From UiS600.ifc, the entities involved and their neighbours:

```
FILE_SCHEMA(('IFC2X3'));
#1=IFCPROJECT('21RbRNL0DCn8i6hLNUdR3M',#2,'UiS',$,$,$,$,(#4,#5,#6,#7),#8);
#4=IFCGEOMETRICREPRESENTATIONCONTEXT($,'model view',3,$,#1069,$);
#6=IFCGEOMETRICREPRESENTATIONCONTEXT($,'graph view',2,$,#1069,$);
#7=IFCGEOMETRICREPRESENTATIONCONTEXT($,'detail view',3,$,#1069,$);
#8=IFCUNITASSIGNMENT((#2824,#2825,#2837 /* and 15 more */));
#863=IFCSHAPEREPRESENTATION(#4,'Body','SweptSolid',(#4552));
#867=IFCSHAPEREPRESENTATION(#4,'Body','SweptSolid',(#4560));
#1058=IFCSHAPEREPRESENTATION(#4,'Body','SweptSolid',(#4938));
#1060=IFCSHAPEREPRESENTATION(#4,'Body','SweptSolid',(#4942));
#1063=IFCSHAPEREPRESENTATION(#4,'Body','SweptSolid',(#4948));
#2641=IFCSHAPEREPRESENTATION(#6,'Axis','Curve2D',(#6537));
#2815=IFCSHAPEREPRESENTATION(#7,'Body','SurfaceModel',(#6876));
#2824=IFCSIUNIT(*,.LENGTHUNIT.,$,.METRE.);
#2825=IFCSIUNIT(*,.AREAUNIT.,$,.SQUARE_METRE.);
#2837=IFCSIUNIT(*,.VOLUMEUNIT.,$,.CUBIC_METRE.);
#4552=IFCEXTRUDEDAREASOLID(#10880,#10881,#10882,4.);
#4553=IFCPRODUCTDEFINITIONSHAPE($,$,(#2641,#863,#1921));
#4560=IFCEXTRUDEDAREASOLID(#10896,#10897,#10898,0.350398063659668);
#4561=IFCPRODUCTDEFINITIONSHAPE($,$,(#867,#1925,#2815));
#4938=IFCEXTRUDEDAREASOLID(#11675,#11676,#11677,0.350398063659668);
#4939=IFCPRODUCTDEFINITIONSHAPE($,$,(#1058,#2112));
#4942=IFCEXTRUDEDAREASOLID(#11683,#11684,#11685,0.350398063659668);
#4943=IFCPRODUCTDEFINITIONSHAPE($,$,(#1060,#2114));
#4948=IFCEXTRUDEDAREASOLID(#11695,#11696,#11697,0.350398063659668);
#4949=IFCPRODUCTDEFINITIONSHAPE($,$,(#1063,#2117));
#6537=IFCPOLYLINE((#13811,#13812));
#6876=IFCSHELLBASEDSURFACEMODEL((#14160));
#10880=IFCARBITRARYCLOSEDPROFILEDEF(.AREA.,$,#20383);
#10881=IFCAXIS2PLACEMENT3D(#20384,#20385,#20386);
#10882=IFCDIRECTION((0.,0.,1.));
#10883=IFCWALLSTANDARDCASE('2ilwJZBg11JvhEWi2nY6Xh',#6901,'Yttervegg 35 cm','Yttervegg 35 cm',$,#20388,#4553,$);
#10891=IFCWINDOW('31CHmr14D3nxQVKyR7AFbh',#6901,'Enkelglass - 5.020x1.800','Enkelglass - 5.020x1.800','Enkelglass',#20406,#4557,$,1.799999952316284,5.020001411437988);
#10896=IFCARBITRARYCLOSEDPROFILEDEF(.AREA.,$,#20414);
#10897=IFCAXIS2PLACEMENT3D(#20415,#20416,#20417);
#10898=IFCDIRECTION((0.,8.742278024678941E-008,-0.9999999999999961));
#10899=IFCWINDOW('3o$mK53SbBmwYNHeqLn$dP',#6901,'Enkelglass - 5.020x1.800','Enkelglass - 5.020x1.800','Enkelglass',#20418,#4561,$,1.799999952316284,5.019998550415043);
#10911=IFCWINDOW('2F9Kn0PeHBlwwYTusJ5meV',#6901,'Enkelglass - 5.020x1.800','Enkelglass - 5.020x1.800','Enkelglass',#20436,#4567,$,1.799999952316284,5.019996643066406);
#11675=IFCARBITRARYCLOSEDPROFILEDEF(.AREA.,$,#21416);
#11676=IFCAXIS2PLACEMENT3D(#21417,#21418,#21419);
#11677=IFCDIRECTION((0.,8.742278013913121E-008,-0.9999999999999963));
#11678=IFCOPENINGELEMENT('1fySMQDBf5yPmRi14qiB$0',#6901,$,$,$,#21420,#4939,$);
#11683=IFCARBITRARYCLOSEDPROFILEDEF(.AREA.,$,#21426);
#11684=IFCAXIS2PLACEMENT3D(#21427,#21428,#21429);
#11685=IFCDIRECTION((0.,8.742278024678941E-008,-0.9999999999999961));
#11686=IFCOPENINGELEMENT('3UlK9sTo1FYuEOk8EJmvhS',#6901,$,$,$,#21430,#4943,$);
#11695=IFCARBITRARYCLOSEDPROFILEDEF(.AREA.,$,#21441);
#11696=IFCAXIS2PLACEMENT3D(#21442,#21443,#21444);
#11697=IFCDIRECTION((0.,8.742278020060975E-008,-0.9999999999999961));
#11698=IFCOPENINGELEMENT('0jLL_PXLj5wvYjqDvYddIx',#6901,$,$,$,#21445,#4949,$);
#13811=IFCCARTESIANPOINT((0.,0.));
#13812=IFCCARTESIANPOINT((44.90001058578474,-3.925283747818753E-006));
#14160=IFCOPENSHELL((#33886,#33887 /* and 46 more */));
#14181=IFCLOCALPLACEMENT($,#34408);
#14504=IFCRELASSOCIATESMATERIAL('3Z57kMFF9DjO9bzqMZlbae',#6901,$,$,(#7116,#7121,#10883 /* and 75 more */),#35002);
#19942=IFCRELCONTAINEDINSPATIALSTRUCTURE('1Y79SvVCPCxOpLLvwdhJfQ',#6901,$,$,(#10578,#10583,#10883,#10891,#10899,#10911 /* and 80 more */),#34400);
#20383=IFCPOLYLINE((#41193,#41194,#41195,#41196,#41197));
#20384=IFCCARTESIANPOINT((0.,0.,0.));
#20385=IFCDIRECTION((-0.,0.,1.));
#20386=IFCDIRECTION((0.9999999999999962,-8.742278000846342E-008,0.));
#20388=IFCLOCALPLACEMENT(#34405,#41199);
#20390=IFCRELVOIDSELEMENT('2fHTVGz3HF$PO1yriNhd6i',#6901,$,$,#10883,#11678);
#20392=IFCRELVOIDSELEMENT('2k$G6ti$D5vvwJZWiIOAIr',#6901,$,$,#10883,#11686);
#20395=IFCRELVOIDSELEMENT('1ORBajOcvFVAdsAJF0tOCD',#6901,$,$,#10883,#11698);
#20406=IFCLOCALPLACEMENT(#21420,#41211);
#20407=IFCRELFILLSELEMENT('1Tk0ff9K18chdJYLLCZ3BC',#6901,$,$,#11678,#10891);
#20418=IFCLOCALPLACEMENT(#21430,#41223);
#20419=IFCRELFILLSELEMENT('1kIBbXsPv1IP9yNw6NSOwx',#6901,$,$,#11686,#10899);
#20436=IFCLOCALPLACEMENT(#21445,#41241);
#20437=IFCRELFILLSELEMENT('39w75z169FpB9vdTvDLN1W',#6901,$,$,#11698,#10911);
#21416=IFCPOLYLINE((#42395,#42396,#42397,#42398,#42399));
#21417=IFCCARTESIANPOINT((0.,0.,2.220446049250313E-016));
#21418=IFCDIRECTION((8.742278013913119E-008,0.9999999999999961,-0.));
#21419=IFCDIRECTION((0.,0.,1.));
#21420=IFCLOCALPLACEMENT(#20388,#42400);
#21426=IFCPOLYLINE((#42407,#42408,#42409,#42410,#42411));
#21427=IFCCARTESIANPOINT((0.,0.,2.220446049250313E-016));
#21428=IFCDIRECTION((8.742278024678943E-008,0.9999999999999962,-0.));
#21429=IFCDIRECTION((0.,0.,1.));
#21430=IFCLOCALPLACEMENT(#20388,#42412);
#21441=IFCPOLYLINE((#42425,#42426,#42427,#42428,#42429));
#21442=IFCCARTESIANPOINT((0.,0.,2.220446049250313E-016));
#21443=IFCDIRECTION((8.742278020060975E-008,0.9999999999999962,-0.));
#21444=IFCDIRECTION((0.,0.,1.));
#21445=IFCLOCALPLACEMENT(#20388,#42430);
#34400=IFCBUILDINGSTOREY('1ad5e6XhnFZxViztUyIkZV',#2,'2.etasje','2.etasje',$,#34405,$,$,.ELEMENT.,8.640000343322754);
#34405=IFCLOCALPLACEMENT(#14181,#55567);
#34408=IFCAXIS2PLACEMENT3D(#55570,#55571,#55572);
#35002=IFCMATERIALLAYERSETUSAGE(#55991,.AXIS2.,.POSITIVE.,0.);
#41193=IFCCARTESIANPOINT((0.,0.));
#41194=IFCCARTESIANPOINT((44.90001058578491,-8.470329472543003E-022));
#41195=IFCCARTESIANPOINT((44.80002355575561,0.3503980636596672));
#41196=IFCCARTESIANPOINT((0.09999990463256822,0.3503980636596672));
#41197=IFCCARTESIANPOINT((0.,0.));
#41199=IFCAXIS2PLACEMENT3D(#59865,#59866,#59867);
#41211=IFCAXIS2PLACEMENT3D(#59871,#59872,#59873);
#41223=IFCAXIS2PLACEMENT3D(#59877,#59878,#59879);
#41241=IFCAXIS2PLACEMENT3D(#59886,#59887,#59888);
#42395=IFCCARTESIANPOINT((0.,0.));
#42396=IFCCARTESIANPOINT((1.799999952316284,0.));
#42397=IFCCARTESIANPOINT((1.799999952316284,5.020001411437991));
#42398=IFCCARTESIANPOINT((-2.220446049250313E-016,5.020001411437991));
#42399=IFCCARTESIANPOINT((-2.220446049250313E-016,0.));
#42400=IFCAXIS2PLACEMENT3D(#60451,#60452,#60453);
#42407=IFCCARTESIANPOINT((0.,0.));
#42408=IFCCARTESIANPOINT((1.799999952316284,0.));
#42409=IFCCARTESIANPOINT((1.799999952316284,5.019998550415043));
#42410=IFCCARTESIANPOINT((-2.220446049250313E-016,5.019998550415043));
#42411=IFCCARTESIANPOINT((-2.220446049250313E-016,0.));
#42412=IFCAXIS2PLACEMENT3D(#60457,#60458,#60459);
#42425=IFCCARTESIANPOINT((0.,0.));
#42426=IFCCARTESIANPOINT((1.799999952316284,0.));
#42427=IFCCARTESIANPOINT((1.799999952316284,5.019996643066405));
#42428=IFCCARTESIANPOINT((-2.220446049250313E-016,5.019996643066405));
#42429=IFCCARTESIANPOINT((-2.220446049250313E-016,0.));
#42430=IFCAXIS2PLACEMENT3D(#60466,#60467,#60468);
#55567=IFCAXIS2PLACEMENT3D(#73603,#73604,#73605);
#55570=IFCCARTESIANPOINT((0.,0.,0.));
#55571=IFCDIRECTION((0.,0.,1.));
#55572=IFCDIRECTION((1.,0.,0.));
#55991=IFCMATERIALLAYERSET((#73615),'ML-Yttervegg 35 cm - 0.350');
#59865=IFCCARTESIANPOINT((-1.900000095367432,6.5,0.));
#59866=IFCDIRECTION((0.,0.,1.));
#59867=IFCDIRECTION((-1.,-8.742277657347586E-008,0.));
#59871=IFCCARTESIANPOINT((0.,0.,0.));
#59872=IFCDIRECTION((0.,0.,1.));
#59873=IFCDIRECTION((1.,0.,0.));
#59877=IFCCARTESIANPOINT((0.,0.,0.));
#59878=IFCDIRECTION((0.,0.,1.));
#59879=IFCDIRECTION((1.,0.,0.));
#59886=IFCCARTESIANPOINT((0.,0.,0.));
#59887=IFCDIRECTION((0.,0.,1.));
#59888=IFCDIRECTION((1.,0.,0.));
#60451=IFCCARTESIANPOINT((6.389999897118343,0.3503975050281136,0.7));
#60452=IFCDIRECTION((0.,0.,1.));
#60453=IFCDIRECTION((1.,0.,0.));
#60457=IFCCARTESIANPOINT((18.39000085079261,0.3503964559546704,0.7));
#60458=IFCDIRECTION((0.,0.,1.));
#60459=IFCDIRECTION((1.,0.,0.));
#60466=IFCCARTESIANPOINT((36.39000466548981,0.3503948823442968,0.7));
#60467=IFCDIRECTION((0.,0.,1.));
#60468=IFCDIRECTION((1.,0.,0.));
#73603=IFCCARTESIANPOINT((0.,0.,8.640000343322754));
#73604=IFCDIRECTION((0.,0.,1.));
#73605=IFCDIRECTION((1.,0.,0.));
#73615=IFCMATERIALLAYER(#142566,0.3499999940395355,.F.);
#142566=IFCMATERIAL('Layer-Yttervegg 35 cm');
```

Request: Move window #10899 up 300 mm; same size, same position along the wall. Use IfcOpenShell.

```python
import numpy as np
import ifcopenshell
import ifcopenshell.api.geometry
import ifcopenshell.util.placement
import ifcopenshell.util.unit

model = ifcopenshell.open("UiS600.ifc")
unit_scale = ifcopenshell.util.unit.calculate_unit_scale(model)

window = model.by_guid("3o$mK53SbBmwYNHeqLn$dP")
opening = window.FillsVoids[0].RelatingOpeningElement
dz = 0.3 / unit_scale

shift = np.array([0.0, 0.0, dz])
# The window is placed relative to its opening, so it follows when the opening moves.
matrix = ifcopenshell.util.placement.get_local_placement(opening.ObjectPlacement)
matrix[:3, 3] += shift
ifcopenshell.api.geometry.edit_object_placement(
    model, product=opening, matrix=matrix, is_si=False, should_transform_children=True
)

print(f"moved by {dz * unit_scale:+.3f} m")

model.write("UiS600_rev.ifc")
```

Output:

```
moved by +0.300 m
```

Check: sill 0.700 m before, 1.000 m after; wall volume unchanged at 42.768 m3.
